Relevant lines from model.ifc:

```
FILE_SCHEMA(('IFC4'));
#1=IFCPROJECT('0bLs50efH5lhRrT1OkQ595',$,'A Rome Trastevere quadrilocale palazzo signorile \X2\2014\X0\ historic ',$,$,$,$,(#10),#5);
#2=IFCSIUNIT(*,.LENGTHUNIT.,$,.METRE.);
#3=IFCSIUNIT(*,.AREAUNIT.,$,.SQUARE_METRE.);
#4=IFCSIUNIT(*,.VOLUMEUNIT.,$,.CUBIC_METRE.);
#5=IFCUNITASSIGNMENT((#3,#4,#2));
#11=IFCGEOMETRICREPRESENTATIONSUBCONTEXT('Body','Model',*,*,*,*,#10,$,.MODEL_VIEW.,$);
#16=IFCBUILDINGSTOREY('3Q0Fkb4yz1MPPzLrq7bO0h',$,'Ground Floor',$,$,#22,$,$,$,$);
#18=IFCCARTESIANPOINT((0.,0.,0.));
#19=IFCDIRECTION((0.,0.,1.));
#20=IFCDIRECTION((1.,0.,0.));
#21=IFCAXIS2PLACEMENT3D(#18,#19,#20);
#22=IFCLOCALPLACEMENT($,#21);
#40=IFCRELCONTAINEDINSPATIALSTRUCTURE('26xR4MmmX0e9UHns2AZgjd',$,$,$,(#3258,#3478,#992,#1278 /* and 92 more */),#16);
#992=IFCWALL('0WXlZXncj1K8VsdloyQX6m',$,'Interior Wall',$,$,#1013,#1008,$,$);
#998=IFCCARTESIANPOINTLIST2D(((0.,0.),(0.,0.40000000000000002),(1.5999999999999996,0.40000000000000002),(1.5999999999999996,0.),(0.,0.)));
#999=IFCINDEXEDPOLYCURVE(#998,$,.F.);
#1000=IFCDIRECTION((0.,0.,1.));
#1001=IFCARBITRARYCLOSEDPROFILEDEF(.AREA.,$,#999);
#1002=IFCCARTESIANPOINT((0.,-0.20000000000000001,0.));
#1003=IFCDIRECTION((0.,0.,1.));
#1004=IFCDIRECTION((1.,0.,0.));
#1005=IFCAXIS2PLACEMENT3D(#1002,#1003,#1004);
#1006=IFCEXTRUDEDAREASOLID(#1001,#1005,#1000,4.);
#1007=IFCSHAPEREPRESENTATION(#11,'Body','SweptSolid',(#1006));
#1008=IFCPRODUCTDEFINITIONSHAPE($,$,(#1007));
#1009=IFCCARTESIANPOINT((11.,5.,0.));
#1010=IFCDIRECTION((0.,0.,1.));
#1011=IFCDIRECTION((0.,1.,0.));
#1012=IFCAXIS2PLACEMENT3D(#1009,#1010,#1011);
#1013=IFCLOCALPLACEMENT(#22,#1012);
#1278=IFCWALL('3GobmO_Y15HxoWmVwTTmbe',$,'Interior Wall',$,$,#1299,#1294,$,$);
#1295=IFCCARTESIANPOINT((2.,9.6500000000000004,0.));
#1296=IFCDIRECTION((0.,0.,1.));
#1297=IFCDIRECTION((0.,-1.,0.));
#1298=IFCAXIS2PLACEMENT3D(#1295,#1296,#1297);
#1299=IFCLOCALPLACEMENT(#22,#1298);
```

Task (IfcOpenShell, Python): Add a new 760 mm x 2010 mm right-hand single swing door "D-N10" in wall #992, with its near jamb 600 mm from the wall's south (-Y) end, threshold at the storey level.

```python
import numpy as np
import ifcopenshell
import ifcopenshell.api.feature
import ifcopenshell.api.geometry
import ifcopenshell.api.root
import ifcopenshell.api.spatial
import ifcopenshell.geom
import ifcopenshell.util.element
import ifcopenshell.util.placement
import ifcopenshell.util.representation
import ifcopenshell.util.shape
import ifcopenshell.util.unit

model = ifcopenshell.open("model.ifc")
unit_scale = ifcopenshell.util.unit.calculate_unit_scale(model)
settings = ifcopenshell.geom.settings()


def volume(element):
    """Net volume in cubic metres, openings subtracted."""
    shape = ifcopenshell.geom.create_shape(settings, element)
    return ifcopenshell.util.shape.get_volume(shape.geometry)


wall = model.by_guid("0WXlZXncj1K8VsdloyQX6m")
storey = ifcopenshell.util.element.get_container(wall, ifc_class="IfcBuildingStorey")
context = ifcopenshell.util.representation.get_context(model, "Model", "Body", "MODEL_VIEW")
before = volume(wall)

width, height, from_end, sill = 0.76, 2.01, 0.6, 0.0  # metres

# The wall runs along its own X axis, and the end named is its -X end.
wall_shape = ifcopenshell.geom.create_shape(settings, wall)
x, y, z = ifcopenshell.util.shape.get_vertices(wall_shape.geometry).T
start = x.min() + from_end
face, thickness = float(y.min()), float(y.max() - y.min())
wall_matrix = ifcopenshell.util.placement.get_local_placement(wall.ObjectPlacement)
level = ifcopenshell.util.placement.get_local_placement(storey.ObjectPlacement)[2, 3]


def in_wall(x, y):
    """Placement at x, y metres in the wall's axes, at sill height."""
    matrix = wall_matrix.copy()
    matrix[:, 3] = wall_matrix @ np.array([x / unit_scale, y / unit_scale, 0.0, 1.0])
    matrix[2, 3] = level + sill / unit_scale
    return matrix


# Opening: a box that overshoots both wall faces by 50 mm.
opening = ifcopenshell.api.root.create_entity(model, ifc_class="IfcOpeningElement", predefined_type="OPENING")
box = ifcopenshell.api.geometry.add_wall_representation(
    model, context=context, length=width, height=height, thickness=thickness + 0.1
)
ifcopenshell.api.geometry.assign_representation(model, product=opening, representation=box)
ifcopenshell.api.geometry.edit_object_placement(model, product=opening, matrix=in_wall(start, face - 0.05), is_si=False)
ifcopenshell.api.feature.add_feature(model, feature=opening, element=wall)

door = ifcopenshell.api.root.create_entity(model, ifc_class="IfcDoor", name="D-N10", predefined_type="DOOR")
door.OverallWidth, door.OverallHeight = width / unit_scale, height / unit_scale
door.OperationType = "SINGLE_SWING_RIGHT"
body = ifcopenshell.api.geometry.add_door_representation(
    model,
    context=context,
    overall_width=door.OverallWidth,
    overall_height=door.OverallHeight,
    operation_type="SINGLE_SWING_RIGHT",
    lining_properties={"LiningDepth": thickness / unit_scale, "ThresholdDepth": thickness / unit_scale},
)
ifcopenshell.api.geometry.assign_representation(model, product=door, representation=body)
ifcopenshell.api.spatial.assign_container(model, products=[door], relating_structure=storey)
ifcopenshell.api.feature.add_filling(model, opening=opening, element=door)

# The lining spans the wall, so the door starts at the wall face.
ifcopenshell.api.geometry.edit_object_placement(model, product=door, matrix=in_wall(start, face), is_si=False)

after = volume(wall)

print(f"wall volume {before:.3f} -> {after:.3f} m3")

model.write("model_v2.ifc")
```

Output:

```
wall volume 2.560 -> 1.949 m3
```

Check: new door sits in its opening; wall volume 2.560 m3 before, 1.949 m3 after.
